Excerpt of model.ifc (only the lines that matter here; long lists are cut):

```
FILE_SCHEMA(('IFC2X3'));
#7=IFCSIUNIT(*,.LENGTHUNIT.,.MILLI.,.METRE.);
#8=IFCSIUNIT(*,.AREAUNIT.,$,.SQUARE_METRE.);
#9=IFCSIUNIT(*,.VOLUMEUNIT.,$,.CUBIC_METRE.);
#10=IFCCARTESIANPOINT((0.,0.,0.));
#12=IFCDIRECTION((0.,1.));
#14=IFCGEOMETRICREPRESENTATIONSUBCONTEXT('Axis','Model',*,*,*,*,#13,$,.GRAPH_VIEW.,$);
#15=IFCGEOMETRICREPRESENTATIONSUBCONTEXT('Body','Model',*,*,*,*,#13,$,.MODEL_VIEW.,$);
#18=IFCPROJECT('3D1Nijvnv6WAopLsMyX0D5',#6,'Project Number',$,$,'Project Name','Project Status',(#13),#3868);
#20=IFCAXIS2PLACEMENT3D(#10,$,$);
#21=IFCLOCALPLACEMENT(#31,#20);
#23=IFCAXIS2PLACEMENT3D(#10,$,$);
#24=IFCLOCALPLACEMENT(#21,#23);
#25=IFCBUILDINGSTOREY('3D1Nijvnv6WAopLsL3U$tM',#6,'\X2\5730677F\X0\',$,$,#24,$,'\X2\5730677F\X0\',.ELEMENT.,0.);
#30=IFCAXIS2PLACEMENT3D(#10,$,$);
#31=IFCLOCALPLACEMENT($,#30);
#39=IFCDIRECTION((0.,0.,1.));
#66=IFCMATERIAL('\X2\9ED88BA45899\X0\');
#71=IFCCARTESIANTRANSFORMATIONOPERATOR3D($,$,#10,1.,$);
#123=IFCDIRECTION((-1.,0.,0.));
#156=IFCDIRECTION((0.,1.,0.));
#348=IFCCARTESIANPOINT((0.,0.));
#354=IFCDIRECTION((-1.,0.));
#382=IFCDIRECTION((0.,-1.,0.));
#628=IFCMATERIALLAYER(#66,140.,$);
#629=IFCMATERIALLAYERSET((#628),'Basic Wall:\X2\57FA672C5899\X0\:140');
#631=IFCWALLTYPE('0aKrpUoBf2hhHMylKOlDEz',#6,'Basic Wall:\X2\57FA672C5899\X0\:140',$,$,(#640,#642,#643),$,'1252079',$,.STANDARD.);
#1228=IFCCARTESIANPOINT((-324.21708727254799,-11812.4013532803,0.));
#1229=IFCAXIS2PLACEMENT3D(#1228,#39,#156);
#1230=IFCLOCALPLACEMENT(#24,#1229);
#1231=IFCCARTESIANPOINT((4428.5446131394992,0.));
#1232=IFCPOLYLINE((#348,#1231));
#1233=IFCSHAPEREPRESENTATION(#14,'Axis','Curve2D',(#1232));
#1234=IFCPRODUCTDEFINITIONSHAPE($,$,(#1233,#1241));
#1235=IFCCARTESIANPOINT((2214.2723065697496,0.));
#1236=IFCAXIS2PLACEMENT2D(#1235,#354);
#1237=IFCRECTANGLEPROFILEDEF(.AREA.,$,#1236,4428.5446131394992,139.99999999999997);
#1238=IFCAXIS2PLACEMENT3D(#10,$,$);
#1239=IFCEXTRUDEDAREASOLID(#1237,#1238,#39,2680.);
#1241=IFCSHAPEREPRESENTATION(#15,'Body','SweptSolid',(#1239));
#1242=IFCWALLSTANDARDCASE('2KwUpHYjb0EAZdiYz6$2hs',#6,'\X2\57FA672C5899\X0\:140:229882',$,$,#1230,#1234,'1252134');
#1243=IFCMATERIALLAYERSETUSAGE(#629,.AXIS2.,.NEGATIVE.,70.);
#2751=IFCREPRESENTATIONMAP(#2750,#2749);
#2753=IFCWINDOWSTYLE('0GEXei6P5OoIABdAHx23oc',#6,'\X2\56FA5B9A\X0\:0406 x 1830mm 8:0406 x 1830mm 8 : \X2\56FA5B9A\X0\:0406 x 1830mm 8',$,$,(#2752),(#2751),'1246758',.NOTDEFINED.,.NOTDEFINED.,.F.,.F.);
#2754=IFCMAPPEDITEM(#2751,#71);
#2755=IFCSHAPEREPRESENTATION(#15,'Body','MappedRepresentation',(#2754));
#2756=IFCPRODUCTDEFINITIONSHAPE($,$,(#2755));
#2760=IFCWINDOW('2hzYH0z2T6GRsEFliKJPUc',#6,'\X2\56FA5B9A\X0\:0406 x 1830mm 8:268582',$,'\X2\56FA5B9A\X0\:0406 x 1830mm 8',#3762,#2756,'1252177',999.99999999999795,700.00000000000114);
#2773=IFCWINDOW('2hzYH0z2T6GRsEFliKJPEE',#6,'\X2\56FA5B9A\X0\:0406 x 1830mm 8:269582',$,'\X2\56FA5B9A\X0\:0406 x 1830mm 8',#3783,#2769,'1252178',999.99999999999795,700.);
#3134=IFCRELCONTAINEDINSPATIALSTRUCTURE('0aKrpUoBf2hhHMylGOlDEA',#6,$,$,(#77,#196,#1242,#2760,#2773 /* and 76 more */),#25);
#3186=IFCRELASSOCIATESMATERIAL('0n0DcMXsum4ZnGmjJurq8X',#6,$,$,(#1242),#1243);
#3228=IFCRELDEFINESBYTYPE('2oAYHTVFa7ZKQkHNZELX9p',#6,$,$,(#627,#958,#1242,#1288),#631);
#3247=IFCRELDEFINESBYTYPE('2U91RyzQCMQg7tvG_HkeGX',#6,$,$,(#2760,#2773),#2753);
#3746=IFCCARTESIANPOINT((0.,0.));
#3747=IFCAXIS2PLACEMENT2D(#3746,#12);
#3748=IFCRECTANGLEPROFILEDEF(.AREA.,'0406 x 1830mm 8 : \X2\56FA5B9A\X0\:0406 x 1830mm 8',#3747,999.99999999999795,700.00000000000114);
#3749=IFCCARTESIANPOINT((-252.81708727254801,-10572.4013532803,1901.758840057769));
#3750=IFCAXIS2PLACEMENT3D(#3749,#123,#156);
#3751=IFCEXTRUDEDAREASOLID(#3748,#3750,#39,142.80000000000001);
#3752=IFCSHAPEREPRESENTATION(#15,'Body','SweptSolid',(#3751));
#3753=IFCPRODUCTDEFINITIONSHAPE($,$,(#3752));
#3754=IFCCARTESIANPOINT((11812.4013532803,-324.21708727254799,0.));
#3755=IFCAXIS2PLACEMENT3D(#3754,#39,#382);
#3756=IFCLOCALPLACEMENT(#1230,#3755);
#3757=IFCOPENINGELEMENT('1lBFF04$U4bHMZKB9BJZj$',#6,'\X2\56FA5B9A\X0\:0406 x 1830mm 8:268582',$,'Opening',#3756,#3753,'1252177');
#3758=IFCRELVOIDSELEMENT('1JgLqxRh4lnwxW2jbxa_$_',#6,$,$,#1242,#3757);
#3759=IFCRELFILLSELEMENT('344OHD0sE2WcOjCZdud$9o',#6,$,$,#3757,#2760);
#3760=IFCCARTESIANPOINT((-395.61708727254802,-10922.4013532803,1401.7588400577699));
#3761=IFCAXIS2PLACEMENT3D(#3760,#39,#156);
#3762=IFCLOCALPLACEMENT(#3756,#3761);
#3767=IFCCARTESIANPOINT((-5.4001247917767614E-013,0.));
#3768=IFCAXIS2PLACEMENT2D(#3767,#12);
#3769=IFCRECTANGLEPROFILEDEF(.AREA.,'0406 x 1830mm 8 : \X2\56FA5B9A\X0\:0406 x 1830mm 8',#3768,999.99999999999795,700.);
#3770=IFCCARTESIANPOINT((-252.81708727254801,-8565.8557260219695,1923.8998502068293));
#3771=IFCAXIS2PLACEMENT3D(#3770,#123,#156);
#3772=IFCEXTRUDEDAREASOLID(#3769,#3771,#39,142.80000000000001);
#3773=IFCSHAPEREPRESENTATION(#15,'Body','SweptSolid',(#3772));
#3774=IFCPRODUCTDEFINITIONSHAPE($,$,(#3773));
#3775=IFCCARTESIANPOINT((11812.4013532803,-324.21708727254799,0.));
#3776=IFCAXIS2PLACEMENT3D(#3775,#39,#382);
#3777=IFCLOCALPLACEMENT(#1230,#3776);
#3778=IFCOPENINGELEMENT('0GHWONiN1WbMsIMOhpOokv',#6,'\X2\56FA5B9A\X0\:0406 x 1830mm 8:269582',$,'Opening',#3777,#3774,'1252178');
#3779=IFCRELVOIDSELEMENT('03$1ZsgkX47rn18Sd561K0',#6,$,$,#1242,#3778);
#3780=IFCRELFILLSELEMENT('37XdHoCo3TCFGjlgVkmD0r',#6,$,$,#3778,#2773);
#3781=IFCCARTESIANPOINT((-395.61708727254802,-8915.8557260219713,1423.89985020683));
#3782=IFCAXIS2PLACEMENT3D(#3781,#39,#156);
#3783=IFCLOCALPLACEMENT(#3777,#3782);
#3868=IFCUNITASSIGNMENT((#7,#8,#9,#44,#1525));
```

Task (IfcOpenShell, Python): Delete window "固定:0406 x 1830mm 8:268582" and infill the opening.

```python
import ifcopenshell
import ifcopenshell.api.feature
import ifcopenshell.api.root
import ifcopenshell.geom
import ifcopenshell.util.shape

model = ifcopenshell.open("model.ifc")
settings = ifcopenshell.geom.settings()


def volume(element):
    """Net volume in cubic metres, openings subtracted."""
    shape = ifcopenshell.geom.create_shape(settings, element)
    return ifcopenshell.util.shape.get_volume(shape.geometry)


window = model.by_id(2760)
opening = window.FillsVoids[0].RelatingOpeningElement
wall = opening.VoidsElements[0].RelatingBuildingElement
before = volume(wall)

ifcopenshell.api.root.remove_product(model, product=window)
ifcopenshell.api.feature.remove_feature(model, feature=opening)

after = volume(wall)

print(f"wall volume {before:.3f} -> {after:.3f} m3")

model.write("model_rev.ifc")
```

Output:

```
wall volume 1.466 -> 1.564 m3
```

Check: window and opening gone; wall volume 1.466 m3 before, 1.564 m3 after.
